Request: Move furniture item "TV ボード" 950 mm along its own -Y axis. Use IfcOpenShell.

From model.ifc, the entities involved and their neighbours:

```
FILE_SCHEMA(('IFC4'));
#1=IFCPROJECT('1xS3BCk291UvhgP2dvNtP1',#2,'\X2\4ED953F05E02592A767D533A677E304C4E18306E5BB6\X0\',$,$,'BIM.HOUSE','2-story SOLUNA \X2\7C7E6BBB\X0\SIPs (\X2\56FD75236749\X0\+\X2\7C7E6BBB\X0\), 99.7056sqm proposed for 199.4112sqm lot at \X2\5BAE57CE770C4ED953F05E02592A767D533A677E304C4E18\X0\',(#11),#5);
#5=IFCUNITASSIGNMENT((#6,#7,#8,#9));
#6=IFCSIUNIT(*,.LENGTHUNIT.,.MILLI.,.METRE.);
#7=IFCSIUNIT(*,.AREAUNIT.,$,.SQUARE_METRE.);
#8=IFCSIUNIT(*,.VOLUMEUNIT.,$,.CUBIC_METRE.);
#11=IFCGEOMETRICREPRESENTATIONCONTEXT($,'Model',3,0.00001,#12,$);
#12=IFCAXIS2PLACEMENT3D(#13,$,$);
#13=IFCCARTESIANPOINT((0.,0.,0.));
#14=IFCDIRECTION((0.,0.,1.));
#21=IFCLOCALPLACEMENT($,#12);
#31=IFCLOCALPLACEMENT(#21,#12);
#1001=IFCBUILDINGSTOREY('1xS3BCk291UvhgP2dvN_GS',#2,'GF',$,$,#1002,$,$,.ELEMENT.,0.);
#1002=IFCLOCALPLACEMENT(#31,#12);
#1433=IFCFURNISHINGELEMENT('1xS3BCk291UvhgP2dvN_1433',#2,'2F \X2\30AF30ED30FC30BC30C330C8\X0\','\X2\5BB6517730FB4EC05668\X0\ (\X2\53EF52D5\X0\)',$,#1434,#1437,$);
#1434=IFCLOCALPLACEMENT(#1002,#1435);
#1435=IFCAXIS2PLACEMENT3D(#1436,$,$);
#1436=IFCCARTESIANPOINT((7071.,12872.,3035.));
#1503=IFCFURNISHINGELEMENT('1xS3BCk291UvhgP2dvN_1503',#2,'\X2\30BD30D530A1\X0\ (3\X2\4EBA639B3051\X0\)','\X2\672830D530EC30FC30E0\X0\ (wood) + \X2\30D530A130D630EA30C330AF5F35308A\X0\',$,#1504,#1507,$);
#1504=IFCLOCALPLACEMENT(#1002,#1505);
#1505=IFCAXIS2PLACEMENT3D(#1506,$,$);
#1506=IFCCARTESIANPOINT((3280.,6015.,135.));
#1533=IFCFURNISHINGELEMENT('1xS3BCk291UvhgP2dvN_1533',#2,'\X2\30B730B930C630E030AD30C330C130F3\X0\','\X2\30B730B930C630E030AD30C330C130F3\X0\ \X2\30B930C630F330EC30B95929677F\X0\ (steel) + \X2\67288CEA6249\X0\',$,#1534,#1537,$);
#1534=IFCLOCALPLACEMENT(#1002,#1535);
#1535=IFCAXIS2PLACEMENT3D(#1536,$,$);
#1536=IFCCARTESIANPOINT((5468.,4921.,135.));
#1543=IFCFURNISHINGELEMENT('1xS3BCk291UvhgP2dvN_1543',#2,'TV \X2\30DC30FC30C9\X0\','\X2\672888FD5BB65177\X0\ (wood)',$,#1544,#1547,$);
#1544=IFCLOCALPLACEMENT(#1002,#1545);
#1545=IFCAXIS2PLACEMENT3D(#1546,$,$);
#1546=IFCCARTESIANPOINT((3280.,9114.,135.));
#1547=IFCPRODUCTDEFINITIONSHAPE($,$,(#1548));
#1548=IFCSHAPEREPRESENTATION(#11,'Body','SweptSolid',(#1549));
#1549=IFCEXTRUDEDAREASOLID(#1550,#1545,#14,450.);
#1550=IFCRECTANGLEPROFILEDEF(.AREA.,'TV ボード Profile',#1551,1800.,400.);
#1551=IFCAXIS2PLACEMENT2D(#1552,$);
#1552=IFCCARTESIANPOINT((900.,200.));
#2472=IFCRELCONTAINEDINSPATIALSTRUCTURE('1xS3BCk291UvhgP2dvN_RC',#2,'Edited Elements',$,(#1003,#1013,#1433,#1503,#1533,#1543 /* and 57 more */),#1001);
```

```python
import ifcopenshell
import ifcopenshell.api.geometry
import ifcopenshell.util.placement
import ifcopenshell.util.unit

model = ifcopenshell.open("model.ifc")
unit_scale = ifcopenshell.util.unit.calculate_unit_scale(model)

item = model.by_guid("1xS3BCk291UvhgP2dvN_1543")
matrix = ifcopenshell.util.placement.get_local_placement(item.ObjectPlacement)
matrix[:3, 3] -= matrix[:3, 1] * 0.95 / unit_scale
ifcopenshell.api.geometry.edit_object_placement(model, product=item, matrix=matrix, is_si=False)

print(ifcopenshell.util.placement.get_local_placement(item.ObjectPlacement).round(3) + 0.0)

model.write("model_v2.ifc")
```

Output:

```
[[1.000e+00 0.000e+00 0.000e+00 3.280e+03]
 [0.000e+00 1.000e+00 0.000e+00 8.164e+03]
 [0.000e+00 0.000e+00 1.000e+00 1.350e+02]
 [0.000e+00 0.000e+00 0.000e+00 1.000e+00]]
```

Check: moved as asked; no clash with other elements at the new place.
